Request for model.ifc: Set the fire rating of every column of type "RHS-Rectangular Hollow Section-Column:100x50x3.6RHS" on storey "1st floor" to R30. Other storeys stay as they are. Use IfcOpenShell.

First a look at what the model holds.

```python
import ifcopenshell
import ifcopenshell.util.element

model = ifcopenshell.open("model.ifc")
print(model.schema)
storey = next(s for s in model.by_type("IfcBuildingStorey") if s.Name == "1st floor")
columns = [e for e in ifcopenshell.util.element.get_decomposition(storey) if e.is_a("IfcColumn")]
seen = {}
for e in columns:
    element_type = ifcopenshell.util.element.get_type(e)
    key = (element_type.Name if element_type != e and element_type else None, ifcopenshell.util.element.get_pset(e, "Pset_ColumnCommon", "FireRating"))
    seen[key] = seen.get(key, 0) + 1
for (name, value), count in sorted(seen.items(), key=str):
    print(count, "x", name, "|", value)
```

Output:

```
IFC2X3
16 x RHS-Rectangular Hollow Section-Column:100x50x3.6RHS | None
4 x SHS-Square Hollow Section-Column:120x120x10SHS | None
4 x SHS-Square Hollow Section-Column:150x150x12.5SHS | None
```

```python
import ifcopenshell
import ifcopenshell.api.pset
import ifcopenshell.util.element

model = ifcopenshell.open("model.ifc")

storey = next(s for s in model.by_type("IfcBuildingStorey") if s.Name == "1st floor")
columns = [e for e in ifcopenshell.util.element.get_decomposition(storey) if e.is_a("IfcColumn")]

count = 0
for e in columns:
    element_type = ifcopenshell.util.element.get_type(e)
    if element_type in (None, e) or element_type.Name != "RHS-Rectangular Hollow Section-Column:100x50x3.6RHS":
        continue
    # add_pset returns the element's existing set when there is one.
    pset = ifcopenshell.api.pset.add_pset(model, product=e, name="Pset_ColumnCommon")
    ifcopenshell.api.pset.edit_pset(model, pset=pset, properties={"FireRating": "R30"})
    count += 1

print(count, "columns updated")

model.write("model_updated.ifc")
```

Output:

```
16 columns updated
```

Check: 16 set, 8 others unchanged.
